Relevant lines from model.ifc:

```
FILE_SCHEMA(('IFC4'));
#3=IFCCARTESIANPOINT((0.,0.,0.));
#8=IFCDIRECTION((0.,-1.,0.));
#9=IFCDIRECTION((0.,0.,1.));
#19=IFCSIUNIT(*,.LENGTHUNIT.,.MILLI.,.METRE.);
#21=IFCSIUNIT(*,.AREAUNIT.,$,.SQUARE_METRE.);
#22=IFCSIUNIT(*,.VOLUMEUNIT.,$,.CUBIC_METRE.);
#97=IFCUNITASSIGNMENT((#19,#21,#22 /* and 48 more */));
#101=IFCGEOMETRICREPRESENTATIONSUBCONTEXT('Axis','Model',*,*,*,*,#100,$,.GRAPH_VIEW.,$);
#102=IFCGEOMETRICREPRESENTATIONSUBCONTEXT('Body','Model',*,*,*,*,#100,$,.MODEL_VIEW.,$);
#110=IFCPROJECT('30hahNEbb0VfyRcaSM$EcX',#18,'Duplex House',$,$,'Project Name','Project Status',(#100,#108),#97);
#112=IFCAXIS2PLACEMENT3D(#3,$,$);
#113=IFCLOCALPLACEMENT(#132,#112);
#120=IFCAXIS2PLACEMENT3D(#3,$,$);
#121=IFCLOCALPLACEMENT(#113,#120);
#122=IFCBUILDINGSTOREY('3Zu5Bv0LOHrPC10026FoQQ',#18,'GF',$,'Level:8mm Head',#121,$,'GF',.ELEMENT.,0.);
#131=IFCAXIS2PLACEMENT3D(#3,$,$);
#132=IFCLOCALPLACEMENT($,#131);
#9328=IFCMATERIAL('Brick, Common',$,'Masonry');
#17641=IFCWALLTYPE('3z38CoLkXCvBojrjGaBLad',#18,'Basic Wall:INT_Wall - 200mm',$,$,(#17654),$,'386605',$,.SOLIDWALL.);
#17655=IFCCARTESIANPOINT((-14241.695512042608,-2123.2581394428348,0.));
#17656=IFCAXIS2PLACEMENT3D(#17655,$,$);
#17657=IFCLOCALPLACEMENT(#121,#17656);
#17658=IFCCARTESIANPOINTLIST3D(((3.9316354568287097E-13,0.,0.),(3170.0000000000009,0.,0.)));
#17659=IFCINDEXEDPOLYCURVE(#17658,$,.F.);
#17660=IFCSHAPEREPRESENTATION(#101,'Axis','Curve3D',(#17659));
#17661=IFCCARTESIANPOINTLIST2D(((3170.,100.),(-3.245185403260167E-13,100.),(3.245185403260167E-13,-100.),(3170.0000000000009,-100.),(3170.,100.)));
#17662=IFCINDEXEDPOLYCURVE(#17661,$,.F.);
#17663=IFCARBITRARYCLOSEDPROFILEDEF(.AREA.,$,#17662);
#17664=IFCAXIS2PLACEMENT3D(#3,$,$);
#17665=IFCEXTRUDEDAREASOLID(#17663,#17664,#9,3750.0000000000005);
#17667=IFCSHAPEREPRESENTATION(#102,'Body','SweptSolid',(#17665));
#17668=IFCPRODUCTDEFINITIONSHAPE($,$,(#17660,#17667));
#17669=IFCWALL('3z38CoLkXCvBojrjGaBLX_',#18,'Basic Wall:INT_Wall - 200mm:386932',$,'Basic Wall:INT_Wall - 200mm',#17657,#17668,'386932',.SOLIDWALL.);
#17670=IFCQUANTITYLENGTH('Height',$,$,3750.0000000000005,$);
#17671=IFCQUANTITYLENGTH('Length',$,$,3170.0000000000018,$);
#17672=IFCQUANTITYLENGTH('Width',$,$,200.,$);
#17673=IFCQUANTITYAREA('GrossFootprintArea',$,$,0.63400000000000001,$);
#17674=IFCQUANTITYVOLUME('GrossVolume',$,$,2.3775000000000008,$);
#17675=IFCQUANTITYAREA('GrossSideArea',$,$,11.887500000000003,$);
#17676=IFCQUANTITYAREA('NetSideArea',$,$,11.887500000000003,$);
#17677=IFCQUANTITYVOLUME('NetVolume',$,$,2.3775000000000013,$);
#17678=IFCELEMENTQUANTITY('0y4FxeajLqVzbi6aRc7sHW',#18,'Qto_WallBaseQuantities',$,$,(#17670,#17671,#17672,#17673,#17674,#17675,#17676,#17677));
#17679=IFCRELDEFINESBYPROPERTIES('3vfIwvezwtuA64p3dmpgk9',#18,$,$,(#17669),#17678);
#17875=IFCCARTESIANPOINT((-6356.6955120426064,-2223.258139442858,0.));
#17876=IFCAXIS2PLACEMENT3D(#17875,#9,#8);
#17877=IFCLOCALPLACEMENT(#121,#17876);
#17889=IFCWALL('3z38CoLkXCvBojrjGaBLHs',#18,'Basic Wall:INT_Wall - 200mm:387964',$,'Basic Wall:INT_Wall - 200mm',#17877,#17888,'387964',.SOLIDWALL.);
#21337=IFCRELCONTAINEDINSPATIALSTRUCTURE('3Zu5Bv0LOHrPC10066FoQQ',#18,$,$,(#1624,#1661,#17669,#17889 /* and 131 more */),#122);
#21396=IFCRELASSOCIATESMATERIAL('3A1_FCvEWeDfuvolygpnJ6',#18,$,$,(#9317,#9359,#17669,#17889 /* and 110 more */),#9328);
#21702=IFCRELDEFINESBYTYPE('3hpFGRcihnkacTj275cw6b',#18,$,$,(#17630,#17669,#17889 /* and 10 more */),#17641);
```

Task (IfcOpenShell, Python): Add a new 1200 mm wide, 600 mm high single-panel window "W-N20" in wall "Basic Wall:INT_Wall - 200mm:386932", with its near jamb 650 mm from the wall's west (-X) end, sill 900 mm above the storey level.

```python
import numpy as np
import ifcopenshell
import ifcopenshell.api.feature
import ifcopenshell.api.geometry
import ifcopenshell.api.pset
import ifcopenshell.api.root
import ifcopenshell.api.spatial
import ifcopenshell.geom
import ifcopenshell.util.element
import ifcopenshell.util.placement
import ifcopenshell.util.representation
import ifcopenshell.util.shape
import ifcopenshell.util.unit

model = ifcopenshell.open("model.ifc")
unit_scale = ifcopenshell.util.unit.calculate_unit_scale(model)
area_scale = ifcopenshell.util.unit.calculate_unit_scale(model, "AREAUNIT")
volume_scale = ifcopenshell.util.unit.calculate_unit_scale(model, "VOLUMEUNIT")
settings = ifcopenshell.geom.settings()


def volume(element):
    """Net volume in cubic metres, openings subtracted."""
    shape = ifcopenshell.geom.create_shape(settings, element)
    return ifcopenshell.util.shape.get_volume(shape.geometry)


wall = model.by_id(17669)
storey = ifcopenshell.util.element.get_container(wall, ifc_class="IfcBuildingStorey")
context = ifcopenshell.util.representation.get_context(model, "Model", "Body", "MODEL_VIEW")
before = volume(wall)

width, height, from_end, sill = 1.2, 0.6, 0.65, 0.9  # metres

# The wall runs along its own X axis, and the end named is its -X end.
wall_shape = ifcopenshell.geom.create_shape(settings, wall)
x, y, z = ifcopenshell.util.shape.get_vertices(wall_shape.geometry).T
start = x.min() + from_end
face, thickness = float(y.min()), float(y.max() - y.min())
wall_matrix = ifcopenshell.util.placement.get_local_placement(wall.ObjectPlacement)
level = ifcopenshell.util.placement.get_local_placement(storey.ObjectPlacement)[2, 3]


def in_wall(x, y):
    """Placement at x, y metres in the wall's axes, at sill height."""
    matrix = wall_matrix.copy()
    matrix[:, 3] = wall_matrix @ np.array([x / unit_scale, y / unit_scale, 0.0, 1.0])
    matrix[2, 3] = level + sill / unit_scale
    return matrix


# Opening: a box that overshoots both wall faces by 50 mm.
opening = ifcopenshell.api.root.create_entity(model, ifc_class="IfcOpeningElement", predefined_type="OPENING")
box = ifcopenshell.api.geometry.add_wall_representation(
    model, context=context, length=width, height=height, thickness=thickness + 0.1
)
ifcopenshell.api.geometry.assign_representation(model, product=opening, representation=box)
ifcopenshell.api.geometry.edit_object_placement(model, product=opening, matrix=in_wall(start, face - 0.05), is_si=False)
ifcopenshell.api.feature.add_feature(model, feature=opening, element=wall)

window = ifcopenshell.api.root.create_entity(model, ifc_class="IfcWindow", name="W-N20", predefined_type="WINDOW")
window.OverallWidth, window.OverallHeight = width / unit_scale, height / unit_scale
window.PartitioningType = "SINGLE_PANEL"
body = ifcopenshell.api.geometry.add_window_representation(
    model,
    context=context,
    overall_width=window.OverallWidth,
    overall_height=window.OverallHeight,
    partition_type="SINGLE_PANEL",
)
ifcopenshell.api.geometry.assign_representation(model, product=window, representation=body)
ifcopenshell.api.spatial.assign_container(model, products=[window], relating_structure=storey)
ifcopenshell.api.feature.add_filling(model, opening=opening, element=window)

# Centre the window in the wall's thickness.
ifcopenshell.api.geometry.edit_object_placement(model, product=window, matrix=in_wall(start, face), is_si=False)
window_shape = ifcopenshell.geom.create_shape(settings, window)
depth = ifcopenshell.util.shape.get_vertices(window_shape.geometry)[:, 1]
offset = face + thickness / 2 - (depth.min() + depth.max()) / 2
ifcopenshell.api.geometry.edit_object_placement(model, product=window, matrix=in_wall(start, offset), is_si=False)

after = volume(wall)

# Update the wall's stored quantities.
qto = model.by_id(ifcopenshell.util.element.get_pset(wall, "Qto_WallBaseQuantities", should_inherit=False)["id"])
ifcopenshell.api.pset.edit_qto(model, qto=qto, properties={
    "NetSideArea": after / thickness / area_scale,
    "NetVolume": after / volume_scale,
})

print(f"wall volume {before:.3f} -> {after:.3f} m3")

model.write("model_rev.ifc")
```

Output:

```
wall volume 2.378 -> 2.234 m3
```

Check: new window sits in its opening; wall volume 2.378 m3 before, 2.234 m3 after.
